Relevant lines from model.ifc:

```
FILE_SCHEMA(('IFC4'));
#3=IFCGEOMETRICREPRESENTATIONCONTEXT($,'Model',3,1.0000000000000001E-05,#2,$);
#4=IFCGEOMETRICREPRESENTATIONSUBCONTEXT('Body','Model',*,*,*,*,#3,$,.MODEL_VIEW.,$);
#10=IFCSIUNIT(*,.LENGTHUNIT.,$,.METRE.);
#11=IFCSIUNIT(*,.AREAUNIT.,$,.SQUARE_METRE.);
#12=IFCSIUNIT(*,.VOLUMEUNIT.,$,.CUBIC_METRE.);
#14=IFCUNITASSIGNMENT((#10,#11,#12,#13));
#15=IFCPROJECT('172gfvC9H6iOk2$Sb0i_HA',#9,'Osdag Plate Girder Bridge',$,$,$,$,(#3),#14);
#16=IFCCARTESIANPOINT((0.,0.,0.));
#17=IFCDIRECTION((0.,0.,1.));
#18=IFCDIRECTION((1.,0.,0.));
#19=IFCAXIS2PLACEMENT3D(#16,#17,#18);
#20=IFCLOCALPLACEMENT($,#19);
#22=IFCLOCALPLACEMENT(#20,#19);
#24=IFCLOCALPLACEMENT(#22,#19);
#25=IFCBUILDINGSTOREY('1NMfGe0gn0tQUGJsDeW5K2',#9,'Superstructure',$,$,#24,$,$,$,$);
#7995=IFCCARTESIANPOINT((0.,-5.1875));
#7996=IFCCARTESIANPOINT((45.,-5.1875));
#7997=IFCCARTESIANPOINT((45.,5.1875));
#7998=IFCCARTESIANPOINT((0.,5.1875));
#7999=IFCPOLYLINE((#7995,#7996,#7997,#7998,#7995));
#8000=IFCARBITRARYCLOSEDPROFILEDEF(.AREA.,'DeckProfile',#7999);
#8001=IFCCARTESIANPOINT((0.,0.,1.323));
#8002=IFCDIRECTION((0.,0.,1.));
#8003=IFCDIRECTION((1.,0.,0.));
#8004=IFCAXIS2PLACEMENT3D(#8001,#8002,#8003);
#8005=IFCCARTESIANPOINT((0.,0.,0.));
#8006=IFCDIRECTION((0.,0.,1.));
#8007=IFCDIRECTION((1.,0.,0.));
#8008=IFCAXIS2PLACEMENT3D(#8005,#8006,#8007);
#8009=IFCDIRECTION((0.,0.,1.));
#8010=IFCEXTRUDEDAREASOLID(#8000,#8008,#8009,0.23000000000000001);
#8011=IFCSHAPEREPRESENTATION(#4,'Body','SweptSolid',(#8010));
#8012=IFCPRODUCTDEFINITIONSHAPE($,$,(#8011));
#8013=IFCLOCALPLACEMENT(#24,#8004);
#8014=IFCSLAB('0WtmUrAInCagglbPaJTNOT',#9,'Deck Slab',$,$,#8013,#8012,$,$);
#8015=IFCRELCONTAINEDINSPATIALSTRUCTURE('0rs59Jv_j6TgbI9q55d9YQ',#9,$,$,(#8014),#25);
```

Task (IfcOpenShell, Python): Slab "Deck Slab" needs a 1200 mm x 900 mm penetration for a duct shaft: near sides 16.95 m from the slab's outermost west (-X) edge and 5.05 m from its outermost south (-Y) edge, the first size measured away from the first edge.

```python
import numpy as np
import ifcopenshell
import ifcopenshell.api.feature
import ifcopenshell.api.geometry
import ifcopenshell.api.root
import ifcopenshell.geom
import ifcopenshell.util.placement
import ifcopenshell.util.representation
import ifcopenshell.util.shape
import ifcopenshell.util.unit

model = ifcopenshell.open("model.ifc")
unit_scale = ifcopenshell.util.unit.calculate_unit_scale(model)
settings = ifcopenshell.geom.settings()


def volume(element):
    """Net volume in cubic metres, openings subtracted."""
    shape = ifcopenshell.geom.create_shape(settings, element)
    return ifcopenshell.util.shape.get_volume(shape.geometry)


slab = model.by_guid("0WtmUrAInCagglbPaJTNOT")
before = volume(slab)

# Extent in the slab's own axes, in metres. The edges named are its -X and -Y sides.
slab_shape = ifcopenshell.geom.create_shape(settings, slab)
vertices = ifcopenshell.util.shape.get_vertices(slab_shape.geometry)
x_min, y_min, bottom = vertices.min(axis=0)
top = vertices[:, 2].max()

opening = ifcopenshell.api.root.create_entity(model, ifc_class="IfcOpeningElement", name="Duct shaft opening", predefined_type="OPENING")
context = ifcopenshell.util.representation.get_context(model, "Model", "Body", "MODEL_VIEW")
width, depth = 1.2, 0.9
outline = [(0.0, 0.0), (width, 0.0), (width, depth), (0.0, depth), (0.0, 0.0)]
# Overshoot both faces by 50 mm so the cut is clean.
shape = ifcopenshell.api.geometry.add_slab_representation(
    model, context=context, depth=top - bottom + 0.1, polyline=outline
)
ifcopenshell.api.geometry.assign_representation(model, product=opening, representation=shape)

matrix = ifcopenshell.util.placement.get_local_placement(slab.ObjectPlacement)
matrix[:, 3] = matrix @ np.append(np.array([x_min + 16.95, y_min + 5.05, bottom - 0.05]) / unit_scale, 1.0)
ifcopenshell.api.geometry.edit_object_placement(model, product=opening, matrix=matrix, is_si=False)
ifcopenshell.api.feature.add_feature(model, feature=opening, element=slab)

after = volume(slab)

print(f"slab volume {before:.3f} -> {after:.3f} m3")

model.write("model-out.ifc")
```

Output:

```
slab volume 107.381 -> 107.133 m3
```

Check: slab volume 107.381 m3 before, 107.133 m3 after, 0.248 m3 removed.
